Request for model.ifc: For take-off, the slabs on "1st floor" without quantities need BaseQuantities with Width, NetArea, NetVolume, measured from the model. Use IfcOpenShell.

First a look at what the model holds.

```python
import ifcopenshell
import ifcopenshell.util.element
import ifcopenshell.util.unit

model = ifcopenshell.open("model.ifc")
print(model.schema)
for unit_type in ("LENGTHUNIT", "AREAUNIT", "VOLUMEUNIT"):
    print(unit_type, ifcopenshell.util.unit.calculate_unit_scale(model, unit_type))
storey = next(s for s in model.by_type("IfcBuildingStorey") if s.Name == "1st floor")
slabs = [e for e in ifcopenshell.util.element.get_decomposition(storey) if e.is_a("IfcSlab")]
for e in sorted(slabs, key=lambda e: e.id()):
    print(e.id(), e.is_a(), e.Name, list(ifcopenshell.util.element.get_psets(e, qtos_only=True)), sep=" | ")
```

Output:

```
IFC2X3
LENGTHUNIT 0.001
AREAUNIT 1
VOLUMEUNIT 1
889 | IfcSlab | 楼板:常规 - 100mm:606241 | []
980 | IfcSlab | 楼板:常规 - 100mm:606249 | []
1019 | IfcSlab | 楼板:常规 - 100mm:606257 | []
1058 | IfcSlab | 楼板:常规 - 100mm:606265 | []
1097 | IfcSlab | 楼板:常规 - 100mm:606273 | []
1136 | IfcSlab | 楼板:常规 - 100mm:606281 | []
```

```python
import ifcopenshell
import ifcopenshell.api.pset
import ifcopenshell.geom
import ifcopenshell.util.element
import ifcopenshell.util.shape
import ifcopenshell.util.unit

model = ifcopenshell.open("model.ifc")
unit_scale = ifcopenshell.util.unit.calculate_unit_scale(model)
area_scale = ifcopenshell.util.unit.calculate_unit_scale(model, "AREAUNIT")
volume_scale = ifcopenshell.util.unit.calculate_unit_scale(model, "VOLUMEUNIT")
settings = ifcopenshell.geom.settings()

storey = next(s for s in model.by_type("IfcBuildingStorey") if s.Name == "1st floor")
slabs = [e for e in ifcopenshell.util.element.get_decomposition(storey) if e.is_a("IfcSlab")]

for e in sorted(slabs, key=lambda e: e.id()):
    if ifcopenshell.util.element.get_psets(e, qtos_only=True, should_inherit=False):
        continue
    # Geometry comes back in metres, in the element's own axes.
    shape = ifcopenshell.geom.create_shape(settings, e)
    values = {
        "Width": ifcopenshell.util.shape.get_z(shape.geometry) / unit_scale,
        "NetArea": ifcopenshell.util.shape.get_footprint_area(shape.geometry) / area_scale,
        "NetVolume": ifcopenshell.util.shape.get_volume(shape.geometry) / volume_scale,
    }
    qto = ifcopenshell.api.pset.add_qto(model, product=e, name="BaseQuantities")
    ifcopenshell.api.pset.edit_qto(model, qto=qto, properties=values)
    print(e.id(), {k: round(v, 3) for k, v in values.items()})

model.write("model_updated.ifc")
```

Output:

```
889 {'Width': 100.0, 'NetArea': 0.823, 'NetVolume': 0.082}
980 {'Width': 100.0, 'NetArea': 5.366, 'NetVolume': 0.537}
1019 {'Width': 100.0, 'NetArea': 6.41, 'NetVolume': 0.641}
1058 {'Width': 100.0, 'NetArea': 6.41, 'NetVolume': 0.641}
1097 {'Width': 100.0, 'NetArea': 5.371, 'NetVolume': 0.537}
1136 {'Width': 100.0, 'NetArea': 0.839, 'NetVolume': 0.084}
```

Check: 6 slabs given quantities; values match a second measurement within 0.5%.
